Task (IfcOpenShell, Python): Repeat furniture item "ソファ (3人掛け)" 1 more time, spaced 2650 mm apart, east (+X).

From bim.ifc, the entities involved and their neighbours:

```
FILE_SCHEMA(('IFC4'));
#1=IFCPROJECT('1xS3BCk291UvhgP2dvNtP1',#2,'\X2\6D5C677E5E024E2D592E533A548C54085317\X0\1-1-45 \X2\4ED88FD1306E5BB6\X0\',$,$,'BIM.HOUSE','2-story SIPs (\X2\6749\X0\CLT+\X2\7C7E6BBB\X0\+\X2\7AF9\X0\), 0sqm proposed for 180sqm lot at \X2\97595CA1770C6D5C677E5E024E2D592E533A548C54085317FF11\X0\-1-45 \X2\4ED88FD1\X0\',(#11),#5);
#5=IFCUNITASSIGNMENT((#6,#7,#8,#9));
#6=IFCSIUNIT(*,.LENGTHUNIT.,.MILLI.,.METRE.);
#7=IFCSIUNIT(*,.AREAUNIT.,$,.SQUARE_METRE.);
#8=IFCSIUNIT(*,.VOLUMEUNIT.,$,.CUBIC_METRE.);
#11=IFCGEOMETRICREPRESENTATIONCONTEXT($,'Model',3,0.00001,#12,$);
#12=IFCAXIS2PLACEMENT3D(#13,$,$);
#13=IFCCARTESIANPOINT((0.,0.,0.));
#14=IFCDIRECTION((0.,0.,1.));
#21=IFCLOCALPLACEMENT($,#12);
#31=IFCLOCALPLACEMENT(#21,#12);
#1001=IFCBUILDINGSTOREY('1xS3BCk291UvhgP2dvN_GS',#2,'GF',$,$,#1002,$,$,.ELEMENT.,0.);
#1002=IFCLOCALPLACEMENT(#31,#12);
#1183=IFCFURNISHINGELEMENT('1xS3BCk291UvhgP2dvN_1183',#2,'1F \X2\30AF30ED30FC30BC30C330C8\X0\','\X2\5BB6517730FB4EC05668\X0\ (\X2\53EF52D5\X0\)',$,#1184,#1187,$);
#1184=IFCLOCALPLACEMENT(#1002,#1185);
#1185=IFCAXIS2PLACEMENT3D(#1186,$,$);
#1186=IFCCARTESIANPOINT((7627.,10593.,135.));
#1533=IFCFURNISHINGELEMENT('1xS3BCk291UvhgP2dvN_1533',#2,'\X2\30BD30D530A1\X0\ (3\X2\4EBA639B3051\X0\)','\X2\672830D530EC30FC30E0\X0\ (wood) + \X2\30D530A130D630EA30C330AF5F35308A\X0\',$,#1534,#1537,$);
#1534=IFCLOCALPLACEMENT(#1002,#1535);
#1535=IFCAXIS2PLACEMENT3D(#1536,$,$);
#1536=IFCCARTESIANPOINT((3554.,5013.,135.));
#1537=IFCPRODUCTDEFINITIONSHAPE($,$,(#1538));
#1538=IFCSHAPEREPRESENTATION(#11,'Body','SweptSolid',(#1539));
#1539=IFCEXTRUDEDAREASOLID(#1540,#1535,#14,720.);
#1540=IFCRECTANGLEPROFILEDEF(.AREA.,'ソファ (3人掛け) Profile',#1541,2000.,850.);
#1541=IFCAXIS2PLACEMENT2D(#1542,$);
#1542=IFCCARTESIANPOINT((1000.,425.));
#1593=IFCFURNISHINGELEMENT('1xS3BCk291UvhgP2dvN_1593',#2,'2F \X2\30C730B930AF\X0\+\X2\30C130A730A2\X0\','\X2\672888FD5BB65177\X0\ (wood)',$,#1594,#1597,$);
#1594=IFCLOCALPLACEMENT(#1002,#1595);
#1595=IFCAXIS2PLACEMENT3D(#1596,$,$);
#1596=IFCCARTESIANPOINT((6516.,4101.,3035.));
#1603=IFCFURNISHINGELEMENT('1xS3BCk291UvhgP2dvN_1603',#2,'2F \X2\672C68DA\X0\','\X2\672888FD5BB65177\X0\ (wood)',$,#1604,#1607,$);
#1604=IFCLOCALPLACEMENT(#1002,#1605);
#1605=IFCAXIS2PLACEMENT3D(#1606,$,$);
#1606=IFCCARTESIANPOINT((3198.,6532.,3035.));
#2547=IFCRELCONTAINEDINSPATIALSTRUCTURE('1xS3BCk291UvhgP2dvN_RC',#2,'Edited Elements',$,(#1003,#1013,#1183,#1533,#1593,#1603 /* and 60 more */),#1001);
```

```python
import numpy as np
import ifcopenshell
import ifcopenshell.api.geometry
import ifcopenshell.api.root
import ifcopenshell.util.element
import ifcopenshell.util.placement

model = ifcopenshell.open("bim.ifc")


def reuse_history(source, copy):
    """copy_class also copies each property set's owner history, people and application; keep the originals."""
    for rel in copy.IsDefinedBy:
        if rel.is_a("IfcRelDefinesByProperties") and (history := rel.RelatingPropertyDefinition.OwnerHistory):
            rel.RelatingPropertyDefinition.OwnerHistory = source.OwnerHistory
            ifcopenshell.util.element.remove_deep2(model, history)


source = model.by_guid("1xS3BCk291UvhgP2dvN_1533")
base = ifcopenshell.util.placement.get_local_placement(source.ObjectPlacement)
step = np.array([1.0, 0.0, 0.0]) * 2650.0

for i in range(1, 2):
    copy = ifcopenshell.api.root.copy_class(model, product=source)
    copy.Representation = ifcopenshell.util.element.copy_deep(
        model, source.Representation, exclude=["IfcGeometricRepresentationContext", "IfcRepresentationMap"]
    )
    reuse_history(source, copy)
    matrix = base.copy()
    matrix[:3, 3] += i * step
    print("added at", matrix[:3, 3].round(3) + 0.0)
    ifcopenshell.api.geometry.edit_object_placement(model, product=copy, matrix=matrix, is_si=False)

model.write("bim_v2.ifc")
```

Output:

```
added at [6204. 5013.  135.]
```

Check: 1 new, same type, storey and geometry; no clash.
